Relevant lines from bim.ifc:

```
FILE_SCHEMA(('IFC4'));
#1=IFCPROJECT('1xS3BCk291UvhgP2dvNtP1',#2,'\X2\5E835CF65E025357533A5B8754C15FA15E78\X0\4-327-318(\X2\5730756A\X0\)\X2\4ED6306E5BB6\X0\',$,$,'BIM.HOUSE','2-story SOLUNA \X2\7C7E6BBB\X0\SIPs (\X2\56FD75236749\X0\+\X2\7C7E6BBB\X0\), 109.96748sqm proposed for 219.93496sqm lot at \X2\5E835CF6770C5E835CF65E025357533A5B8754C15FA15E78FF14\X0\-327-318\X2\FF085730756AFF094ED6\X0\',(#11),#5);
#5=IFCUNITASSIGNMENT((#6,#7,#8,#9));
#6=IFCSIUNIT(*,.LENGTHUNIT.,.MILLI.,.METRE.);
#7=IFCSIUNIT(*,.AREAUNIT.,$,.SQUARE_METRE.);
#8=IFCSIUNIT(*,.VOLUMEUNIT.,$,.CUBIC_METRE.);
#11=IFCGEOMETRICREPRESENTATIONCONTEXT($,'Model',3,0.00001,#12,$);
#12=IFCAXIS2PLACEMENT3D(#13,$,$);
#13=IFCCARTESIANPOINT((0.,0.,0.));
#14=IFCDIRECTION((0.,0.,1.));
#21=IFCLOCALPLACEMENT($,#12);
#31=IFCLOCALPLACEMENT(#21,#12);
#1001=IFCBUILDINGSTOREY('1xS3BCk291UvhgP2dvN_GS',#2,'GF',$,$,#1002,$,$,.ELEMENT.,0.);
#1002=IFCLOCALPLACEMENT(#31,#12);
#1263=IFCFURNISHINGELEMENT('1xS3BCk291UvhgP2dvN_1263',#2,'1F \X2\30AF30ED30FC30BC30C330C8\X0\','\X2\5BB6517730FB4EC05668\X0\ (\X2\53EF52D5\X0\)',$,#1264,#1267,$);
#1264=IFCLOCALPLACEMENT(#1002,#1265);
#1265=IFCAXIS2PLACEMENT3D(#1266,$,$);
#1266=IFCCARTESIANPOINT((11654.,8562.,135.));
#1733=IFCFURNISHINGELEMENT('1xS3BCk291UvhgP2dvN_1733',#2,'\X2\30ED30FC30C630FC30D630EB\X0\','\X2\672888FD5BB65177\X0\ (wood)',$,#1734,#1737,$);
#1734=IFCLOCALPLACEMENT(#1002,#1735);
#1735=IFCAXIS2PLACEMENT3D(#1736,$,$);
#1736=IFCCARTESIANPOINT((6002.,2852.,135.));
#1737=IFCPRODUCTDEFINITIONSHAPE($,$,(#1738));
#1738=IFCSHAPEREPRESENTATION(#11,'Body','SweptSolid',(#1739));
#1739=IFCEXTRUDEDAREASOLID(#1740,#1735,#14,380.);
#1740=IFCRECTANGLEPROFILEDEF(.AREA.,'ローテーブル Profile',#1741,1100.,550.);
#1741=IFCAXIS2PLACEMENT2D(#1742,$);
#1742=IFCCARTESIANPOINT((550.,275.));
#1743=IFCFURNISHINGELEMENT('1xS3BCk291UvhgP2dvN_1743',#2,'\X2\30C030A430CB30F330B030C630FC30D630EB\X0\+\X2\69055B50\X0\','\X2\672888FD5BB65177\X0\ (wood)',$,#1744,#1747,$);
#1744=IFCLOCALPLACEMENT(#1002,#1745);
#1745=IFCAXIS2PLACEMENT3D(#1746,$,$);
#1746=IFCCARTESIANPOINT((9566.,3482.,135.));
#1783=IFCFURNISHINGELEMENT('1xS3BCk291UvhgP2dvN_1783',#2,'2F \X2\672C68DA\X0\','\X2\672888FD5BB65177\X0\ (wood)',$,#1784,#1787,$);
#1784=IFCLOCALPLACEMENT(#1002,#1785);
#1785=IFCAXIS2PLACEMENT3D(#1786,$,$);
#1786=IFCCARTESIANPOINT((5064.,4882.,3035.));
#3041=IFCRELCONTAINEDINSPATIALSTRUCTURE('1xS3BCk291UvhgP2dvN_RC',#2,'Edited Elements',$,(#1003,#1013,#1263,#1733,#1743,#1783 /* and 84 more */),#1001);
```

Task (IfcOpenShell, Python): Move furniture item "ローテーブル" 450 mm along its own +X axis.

```python
import ifcopenshell
import ifcopenshell.api.geometry
import ifcopenshell.util.placement
import ifcopenshell.util.unit

model = ifcopenshell.open("bim.ifc")
unit_scale = ifcopenshell.util.unit.calculate_unit_scale(model)

item = model.by_guid("1xS3BCk291UvhgP2dvN_1733")
matrix = ifcopenshell.util.placement.get_local_placement(item.ObjectPlacement)
matrix[:3, 3] += matrix[:3, 0] * 0.45 / unit_scale
ifcopenshell.api.geometry.edit_object_placement(model, product=item, matrix=matrix, is_si=False)

print(ifcopenshell.util.placement.get_local_placement(item.ObjectPlacement).round(3) + 0.0)

model.write("bim-out.ifc")
```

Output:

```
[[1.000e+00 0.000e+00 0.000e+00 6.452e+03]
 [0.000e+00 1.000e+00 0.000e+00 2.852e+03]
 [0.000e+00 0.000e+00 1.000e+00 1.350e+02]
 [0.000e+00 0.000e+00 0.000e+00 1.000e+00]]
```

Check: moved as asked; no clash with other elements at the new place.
